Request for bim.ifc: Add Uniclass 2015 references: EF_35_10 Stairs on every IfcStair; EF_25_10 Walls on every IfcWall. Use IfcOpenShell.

First a look at what the model holds.

```python
import ifcopenshell

model = ifcopenshell.open("bim.ifc")
print(model.schema)
print("classifications:", [c.Name for c in model.by_type("IfcClassification")])
for ifc_class in ("IfcDoor", "IfcRoof", "IfcStair", "IfcWall", "IfcWindow"):
    print(ifc_class, len(model.by_type(ifc_class)))
```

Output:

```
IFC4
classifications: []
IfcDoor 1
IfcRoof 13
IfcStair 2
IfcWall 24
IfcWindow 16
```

```python
import ifcopenshell
import ifcopenshell.api.classification

model = ifcopenshell.open("bim.ifc")

system = ifcopenshell.api.classification.add_classification(model, classification="Uniclass 2015")

codes = {
    "IfcStair": ("EF_35_10", "Stairs"),
    "IfcWall": ("EF_25_10", "Walls"),
}
for ifc_class, (code, name) in codes.items():
    products = model.by_type(ifc_class)
    ifcopenshell.api.classification.add_reference(
        model, products=products, classification=system, identification=code, name=name
    )
    print(code, len(products))

model.write("bim_rev.ifc")
```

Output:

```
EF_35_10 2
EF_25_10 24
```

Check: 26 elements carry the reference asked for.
